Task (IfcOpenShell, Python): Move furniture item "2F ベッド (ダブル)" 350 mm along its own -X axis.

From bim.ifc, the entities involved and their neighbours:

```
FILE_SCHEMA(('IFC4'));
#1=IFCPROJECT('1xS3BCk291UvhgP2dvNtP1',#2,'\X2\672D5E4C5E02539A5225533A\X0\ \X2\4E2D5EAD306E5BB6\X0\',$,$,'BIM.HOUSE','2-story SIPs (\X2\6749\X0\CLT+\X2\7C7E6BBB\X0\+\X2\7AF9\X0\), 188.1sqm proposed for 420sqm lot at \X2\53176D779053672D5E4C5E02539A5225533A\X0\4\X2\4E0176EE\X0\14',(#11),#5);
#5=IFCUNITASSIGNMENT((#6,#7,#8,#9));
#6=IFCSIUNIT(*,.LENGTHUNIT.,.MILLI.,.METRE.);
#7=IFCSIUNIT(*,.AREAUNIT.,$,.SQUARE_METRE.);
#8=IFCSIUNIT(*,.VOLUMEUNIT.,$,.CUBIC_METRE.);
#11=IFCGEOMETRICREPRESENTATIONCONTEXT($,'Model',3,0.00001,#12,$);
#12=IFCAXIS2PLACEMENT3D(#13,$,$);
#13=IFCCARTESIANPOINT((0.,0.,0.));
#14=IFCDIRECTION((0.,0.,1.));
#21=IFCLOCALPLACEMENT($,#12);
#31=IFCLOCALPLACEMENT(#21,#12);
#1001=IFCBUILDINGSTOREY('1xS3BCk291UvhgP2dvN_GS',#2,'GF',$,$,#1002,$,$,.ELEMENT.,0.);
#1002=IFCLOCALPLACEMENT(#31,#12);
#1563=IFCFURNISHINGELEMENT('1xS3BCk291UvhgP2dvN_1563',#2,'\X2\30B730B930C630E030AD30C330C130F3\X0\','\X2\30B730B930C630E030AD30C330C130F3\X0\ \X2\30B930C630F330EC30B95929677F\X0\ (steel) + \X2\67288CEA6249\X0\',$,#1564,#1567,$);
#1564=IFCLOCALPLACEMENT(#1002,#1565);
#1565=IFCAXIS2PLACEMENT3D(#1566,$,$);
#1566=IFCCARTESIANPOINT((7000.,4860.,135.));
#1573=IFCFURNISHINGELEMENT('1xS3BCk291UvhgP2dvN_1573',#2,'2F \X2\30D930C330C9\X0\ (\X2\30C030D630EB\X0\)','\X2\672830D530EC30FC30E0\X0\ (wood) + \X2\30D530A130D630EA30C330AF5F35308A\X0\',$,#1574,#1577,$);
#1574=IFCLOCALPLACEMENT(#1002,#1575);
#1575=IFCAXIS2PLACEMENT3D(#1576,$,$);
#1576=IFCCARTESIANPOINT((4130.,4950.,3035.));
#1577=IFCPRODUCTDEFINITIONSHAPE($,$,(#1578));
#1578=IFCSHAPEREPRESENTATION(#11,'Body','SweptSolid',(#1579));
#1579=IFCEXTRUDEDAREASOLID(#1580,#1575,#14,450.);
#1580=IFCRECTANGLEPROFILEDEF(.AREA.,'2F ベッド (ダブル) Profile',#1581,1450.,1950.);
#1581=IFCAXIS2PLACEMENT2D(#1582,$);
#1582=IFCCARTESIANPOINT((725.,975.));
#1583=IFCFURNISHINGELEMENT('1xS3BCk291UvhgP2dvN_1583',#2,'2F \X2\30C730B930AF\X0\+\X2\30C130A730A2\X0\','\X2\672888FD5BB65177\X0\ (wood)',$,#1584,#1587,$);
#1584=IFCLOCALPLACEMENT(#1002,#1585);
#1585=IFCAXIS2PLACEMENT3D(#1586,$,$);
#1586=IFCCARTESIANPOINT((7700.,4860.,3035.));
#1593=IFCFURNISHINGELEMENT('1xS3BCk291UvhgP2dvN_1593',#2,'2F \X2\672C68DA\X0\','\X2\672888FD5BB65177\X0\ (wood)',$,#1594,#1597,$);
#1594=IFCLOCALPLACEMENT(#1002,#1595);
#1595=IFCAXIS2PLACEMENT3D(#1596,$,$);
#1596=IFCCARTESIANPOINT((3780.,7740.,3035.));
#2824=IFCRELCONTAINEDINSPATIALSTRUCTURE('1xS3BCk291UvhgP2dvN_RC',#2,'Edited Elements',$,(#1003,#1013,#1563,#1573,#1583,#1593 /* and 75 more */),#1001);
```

```python
import ifcopenshell
import ifcopenshell.api.geometry
import ifcopenshell.util.placement
import ifcopenshell.util.unit

model = ifcopenshell.open("bim.ifc")
unit_scale = ifcopenshell.util.unit.calculate_unit_scale(model)

item = model.by_guid("1xS3BCk291UvhgP2dvN_1573")
matrix = ifcopenshell.util.placement.get_local_placement(item.ObjectPlacement)
matrix[:3, 3] -= matrix[:3, 0] * 0.35 / unit_scale
ifcopenshell.api.geometry.edit_object_placement(model, product=item, matrix=matrix, is_si=False)

print(ifcopenshell.util.placement.get_local_placement(item.ObjectPlacement).round(3) + 0.0)

model.write("bim_updated.ifc")
```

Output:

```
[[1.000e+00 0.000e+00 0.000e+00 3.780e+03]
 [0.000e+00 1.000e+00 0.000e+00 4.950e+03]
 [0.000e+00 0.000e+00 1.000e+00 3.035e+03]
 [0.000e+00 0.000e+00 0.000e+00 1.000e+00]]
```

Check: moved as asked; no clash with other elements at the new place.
